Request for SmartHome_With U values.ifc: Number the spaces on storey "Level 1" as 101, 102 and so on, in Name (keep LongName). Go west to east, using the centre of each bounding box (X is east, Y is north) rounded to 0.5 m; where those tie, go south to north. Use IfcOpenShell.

First a look at what the model holds.

```python
import ifcopenshell
import ifcopenshell.util.element
import ifcopenshell.util.placement

model = ifcopenshell.open("SmartHome_With U values.ifc")
print(model.schema)
storey = next(s for s in model.by_type("IfcBuildingStorey") if s.Name == "Level 1")
spaces = [e for e in ifcopenshell.util.element.get_decomposition(storey) if e.is_a("IfcSpace")]
for e in sorted(spaces, key=lambda e: e.id()):
    origin = ifcopenshell.util.placement.get_local_placement(e.ObjectPlacement)[:3, 3]
    print(e.id(), e.Name, e.LongName, origin.round(2) + 0.0, sep=" | ")
```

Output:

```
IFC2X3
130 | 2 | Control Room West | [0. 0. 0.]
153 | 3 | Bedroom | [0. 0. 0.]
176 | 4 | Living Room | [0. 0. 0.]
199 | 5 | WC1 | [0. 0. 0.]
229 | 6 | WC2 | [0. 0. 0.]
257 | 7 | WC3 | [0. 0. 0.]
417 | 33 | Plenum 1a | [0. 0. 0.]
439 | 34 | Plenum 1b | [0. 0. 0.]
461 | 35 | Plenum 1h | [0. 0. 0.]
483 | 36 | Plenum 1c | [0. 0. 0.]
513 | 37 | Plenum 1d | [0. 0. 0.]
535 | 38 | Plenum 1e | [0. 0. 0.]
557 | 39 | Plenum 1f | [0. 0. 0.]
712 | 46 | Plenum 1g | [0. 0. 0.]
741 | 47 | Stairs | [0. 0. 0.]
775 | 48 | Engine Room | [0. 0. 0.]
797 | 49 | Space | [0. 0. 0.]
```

```python
import ifcopenshell
import ifcopenshell.geom
import ifcopenshell.util.element
import ifcopenshell.util.shape

model = ifcopenshell.open("SmartHome_With U values.ifc")
settings = ifcopenshell.geom.settings()
settings.set("use-world-coords", True)


def centre(element):
    shape = ifcopenshell.geom.create_shape(settings, element)
    return ifcopenshell.util.shape.get_bbox_centroid(shape.geometry)


storey = next(s for s in model.by_type("IfcBuildingStorey") if s.Name == "Level 1")
spaces = [e for e in ifcopenshell.util.element.get_decomposition(storey) if e.is_a("IfcSpace")]

# Insertion points can sit at a corner or the storey origin, so sort by the geometry (in metres).
centres = {e: centre(e) for e in spaces}
spaces.sort(key=lambda e: (round(centres[e][0] / 0.5), centres[e][1]))

for i, e in enumerate(spaces, start=1):
    number = f"1{i:02d}"
    e.Name = number
    print(e.id(), number)

model.write("SmartHome_With U values_updated.ifc")
```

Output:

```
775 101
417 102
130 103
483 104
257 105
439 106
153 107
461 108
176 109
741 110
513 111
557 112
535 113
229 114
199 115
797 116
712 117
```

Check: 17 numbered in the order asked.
